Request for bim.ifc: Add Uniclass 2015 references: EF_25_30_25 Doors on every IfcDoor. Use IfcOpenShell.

First a look at what the model holds.

```python
import ifcopenshell

model = ifcopenshell.open("bim.ifc")
print(model.schema)
print("classifications:", [c.Name for c in model.by_type("IfcClassification")])
for ifc_class in ("IfcDoor", "IfcRoof", "IfcStair", "IfcWall", "IfcWindow"):
    print(ifc_class, len(model.by_type(ifc_class)))
```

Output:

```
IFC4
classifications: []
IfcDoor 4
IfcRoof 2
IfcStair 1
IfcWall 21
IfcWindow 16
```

```python
import ifcopenshell
import ifcopenshell.api.classification

model = ifcopenshell.open("bim.ifc")

system = ifcopenshell.api.classification.add_classification(model, classification="Uniclass 2015")

codes = {
    "IfcDoor": ("EF_25_30_25", "Doors"),
}
for ifc_class, (code, name) in codes.items():
    products = model.by_type(ifc_class)
    ifcopenshell.api.classification.add_reference(
        model, products=products, classification=system, identification=code, name=name
    )
    print(code, len(products))

model.write("bim-out.ifc")
```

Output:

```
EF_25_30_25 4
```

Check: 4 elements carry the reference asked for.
